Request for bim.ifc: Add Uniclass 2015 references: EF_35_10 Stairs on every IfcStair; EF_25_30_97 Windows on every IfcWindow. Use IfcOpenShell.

First a look at what the model holds.

```python
import ifcopenshell

model = ifcopenshell.open("bim.ifc")
print(model.schema)
print("classifications:", [c.Name for c in model.by_type("IfcClassification")])
for ifc_class in ("IfcDoor", "IfcRoof", "IfcStair", "IfcWall", "IfcWindow"):
    print(ifc_class, len(model.by_type(ifc_class)))
```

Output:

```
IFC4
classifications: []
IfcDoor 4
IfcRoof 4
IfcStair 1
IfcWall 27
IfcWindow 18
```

```python
import ifcopenshell
import ifcopenshell.api.classification

model = ifcopenshell.open("bim.ifc")

system = ifcopenshell.api.classification.add_classification(model, classification="Uniclass 2015")

codes = {
    "IfcStair": ("EF_35_10", "Stairs"),
    "IfcWindow": ("EF_25_30_97", "Windows"),
}
for ifc_class, (code, name) in codes.items():
    products = model.by_type(ifc_class)
    ifcopenshell.api.classification.add_reference(
        model, products=products, classification=system, identification=code, name=name
    )
    print(code, len(products))

model.write("bim_edited.ifc")
```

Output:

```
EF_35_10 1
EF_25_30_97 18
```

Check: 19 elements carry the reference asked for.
